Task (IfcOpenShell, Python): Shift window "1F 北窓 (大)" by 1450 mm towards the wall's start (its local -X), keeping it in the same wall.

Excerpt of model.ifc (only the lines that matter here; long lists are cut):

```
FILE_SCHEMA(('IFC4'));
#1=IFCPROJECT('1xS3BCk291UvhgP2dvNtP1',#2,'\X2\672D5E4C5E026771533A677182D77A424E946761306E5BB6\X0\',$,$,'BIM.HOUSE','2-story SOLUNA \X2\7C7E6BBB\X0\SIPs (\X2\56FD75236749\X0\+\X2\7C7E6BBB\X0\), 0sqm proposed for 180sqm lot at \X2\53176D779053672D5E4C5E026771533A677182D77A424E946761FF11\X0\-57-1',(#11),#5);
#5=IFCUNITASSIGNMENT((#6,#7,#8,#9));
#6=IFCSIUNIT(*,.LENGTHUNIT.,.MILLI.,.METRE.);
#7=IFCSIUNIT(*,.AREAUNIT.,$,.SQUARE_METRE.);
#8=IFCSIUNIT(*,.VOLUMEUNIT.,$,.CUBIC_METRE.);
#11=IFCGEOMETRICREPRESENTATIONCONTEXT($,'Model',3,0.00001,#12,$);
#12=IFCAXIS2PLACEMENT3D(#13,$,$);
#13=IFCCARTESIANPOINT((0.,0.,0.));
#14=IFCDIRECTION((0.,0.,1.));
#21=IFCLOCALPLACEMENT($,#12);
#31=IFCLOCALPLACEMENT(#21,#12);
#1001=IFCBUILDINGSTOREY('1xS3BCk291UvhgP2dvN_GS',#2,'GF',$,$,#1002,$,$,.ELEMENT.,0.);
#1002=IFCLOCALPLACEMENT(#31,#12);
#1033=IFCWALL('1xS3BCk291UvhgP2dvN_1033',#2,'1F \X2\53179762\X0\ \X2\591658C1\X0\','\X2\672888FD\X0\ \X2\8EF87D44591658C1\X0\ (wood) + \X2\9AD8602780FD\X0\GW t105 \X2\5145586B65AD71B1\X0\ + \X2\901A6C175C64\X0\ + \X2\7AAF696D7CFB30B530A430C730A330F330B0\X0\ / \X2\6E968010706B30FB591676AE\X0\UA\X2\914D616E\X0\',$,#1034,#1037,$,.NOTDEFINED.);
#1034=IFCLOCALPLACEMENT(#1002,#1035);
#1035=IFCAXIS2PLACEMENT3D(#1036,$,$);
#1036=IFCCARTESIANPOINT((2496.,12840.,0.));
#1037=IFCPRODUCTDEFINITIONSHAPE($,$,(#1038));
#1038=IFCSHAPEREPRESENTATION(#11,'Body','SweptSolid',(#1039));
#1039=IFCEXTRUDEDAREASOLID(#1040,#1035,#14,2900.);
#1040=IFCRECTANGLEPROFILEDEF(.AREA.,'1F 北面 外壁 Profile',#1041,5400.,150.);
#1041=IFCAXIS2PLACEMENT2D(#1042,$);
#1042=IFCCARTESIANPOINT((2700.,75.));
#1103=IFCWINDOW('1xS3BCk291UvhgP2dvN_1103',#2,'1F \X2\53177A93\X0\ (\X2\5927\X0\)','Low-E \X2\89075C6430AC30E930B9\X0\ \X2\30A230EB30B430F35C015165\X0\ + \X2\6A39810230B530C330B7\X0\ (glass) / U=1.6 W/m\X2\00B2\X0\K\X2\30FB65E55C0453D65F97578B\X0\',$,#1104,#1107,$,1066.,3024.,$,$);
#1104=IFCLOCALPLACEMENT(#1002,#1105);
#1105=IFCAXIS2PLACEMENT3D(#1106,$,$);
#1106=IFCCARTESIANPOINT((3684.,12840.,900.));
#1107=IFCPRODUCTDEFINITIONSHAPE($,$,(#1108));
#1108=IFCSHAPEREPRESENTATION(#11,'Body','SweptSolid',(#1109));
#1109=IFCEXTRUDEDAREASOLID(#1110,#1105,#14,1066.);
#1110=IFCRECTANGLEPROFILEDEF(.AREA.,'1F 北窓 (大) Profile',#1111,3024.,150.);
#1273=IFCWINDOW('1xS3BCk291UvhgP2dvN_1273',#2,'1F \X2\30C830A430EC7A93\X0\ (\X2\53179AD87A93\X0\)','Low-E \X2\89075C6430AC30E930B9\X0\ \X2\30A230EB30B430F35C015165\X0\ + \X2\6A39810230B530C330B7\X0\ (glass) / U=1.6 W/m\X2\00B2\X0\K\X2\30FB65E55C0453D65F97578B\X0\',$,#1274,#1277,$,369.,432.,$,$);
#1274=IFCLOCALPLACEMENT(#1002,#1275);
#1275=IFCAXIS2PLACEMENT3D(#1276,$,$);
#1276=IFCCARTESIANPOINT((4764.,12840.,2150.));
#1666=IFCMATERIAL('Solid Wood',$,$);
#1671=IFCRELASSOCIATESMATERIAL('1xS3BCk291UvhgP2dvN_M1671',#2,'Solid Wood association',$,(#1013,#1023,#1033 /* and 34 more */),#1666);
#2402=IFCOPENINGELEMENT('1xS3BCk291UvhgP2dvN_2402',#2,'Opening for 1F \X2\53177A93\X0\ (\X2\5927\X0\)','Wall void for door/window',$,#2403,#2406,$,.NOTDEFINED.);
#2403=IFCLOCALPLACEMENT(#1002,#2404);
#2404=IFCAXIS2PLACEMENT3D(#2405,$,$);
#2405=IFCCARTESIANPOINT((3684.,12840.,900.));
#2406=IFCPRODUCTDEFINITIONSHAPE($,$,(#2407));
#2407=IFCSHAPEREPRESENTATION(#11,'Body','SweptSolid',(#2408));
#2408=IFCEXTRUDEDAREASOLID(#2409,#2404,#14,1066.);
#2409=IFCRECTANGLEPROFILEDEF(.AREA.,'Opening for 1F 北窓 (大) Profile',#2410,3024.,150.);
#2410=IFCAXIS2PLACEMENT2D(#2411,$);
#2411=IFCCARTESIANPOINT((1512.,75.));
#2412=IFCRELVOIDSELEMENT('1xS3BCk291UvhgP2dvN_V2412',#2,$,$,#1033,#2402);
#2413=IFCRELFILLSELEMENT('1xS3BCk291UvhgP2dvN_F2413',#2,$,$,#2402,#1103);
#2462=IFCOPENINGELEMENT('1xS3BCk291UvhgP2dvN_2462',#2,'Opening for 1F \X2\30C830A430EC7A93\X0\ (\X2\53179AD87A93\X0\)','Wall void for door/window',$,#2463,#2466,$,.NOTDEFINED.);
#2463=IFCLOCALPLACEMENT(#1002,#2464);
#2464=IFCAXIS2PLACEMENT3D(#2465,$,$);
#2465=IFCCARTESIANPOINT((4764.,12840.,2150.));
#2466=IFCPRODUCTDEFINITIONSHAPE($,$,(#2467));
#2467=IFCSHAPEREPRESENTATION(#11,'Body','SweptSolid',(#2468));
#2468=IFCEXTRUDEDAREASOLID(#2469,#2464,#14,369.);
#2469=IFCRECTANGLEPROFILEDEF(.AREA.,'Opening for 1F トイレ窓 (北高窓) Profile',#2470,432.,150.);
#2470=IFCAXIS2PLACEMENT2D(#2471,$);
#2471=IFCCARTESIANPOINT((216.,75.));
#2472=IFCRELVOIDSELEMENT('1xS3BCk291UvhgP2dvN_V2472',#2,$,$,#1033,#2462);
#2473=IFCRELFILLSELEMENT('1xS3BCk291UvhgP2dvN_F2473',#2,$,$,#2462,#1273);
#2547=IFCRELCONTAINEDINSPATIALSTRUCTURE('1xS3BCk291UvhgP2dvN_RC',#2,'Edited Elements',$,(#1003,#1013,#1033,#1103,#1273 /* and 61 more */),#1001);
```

```python
import ifcopenshell
import ifcopenshell.api.geometry
import ifcopenshell.util.placement
import ifcopenshell.util.unit

model = ifcopenshell.open("model.ifc")
unit_scale = ifcopenshell.util.unit.calculate_unit_scale(model)

window = model.by_guid("1xS3BCk291UvhgP2dvN_1103")
opening = window.FillsVoids[0].RelatingOpeningElement
wall = opening.VoidsElements[0].RelatingBuildingElement

wall_matrix = ifcopenshell.util.placement.get_local_placement(wall.ObjectPlacement)
shift = wall_matrix[:3, 0] * -1.45 / unit_scale
before = ifcopenshell.util.placement.get_local_placement(window.ObjectPlacement)[:3, 3].copy()

# The window is not placed relative to its opening, so move both.
for product in (opening, window):
    matrix = ifcopenshell.util.placement.get_local_placement(product.ObjectPlacement)
    matrix[:3, 3] += shift
    ifcopenshell.api.geometry.edit_object_placement(model, product=product, matrix=matrix, is_si=False)

after = ifcopenshell.util.placement.get_local_placement(window.ObjectPlacement)[:3, 3]
print("window moved by", (after - before).round(3) + 0.0)

model.write("model_updated.ifc")
```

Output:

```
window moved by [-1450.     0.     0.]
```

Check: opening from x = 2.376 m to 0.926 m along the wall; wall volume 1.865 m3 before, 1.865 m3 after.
